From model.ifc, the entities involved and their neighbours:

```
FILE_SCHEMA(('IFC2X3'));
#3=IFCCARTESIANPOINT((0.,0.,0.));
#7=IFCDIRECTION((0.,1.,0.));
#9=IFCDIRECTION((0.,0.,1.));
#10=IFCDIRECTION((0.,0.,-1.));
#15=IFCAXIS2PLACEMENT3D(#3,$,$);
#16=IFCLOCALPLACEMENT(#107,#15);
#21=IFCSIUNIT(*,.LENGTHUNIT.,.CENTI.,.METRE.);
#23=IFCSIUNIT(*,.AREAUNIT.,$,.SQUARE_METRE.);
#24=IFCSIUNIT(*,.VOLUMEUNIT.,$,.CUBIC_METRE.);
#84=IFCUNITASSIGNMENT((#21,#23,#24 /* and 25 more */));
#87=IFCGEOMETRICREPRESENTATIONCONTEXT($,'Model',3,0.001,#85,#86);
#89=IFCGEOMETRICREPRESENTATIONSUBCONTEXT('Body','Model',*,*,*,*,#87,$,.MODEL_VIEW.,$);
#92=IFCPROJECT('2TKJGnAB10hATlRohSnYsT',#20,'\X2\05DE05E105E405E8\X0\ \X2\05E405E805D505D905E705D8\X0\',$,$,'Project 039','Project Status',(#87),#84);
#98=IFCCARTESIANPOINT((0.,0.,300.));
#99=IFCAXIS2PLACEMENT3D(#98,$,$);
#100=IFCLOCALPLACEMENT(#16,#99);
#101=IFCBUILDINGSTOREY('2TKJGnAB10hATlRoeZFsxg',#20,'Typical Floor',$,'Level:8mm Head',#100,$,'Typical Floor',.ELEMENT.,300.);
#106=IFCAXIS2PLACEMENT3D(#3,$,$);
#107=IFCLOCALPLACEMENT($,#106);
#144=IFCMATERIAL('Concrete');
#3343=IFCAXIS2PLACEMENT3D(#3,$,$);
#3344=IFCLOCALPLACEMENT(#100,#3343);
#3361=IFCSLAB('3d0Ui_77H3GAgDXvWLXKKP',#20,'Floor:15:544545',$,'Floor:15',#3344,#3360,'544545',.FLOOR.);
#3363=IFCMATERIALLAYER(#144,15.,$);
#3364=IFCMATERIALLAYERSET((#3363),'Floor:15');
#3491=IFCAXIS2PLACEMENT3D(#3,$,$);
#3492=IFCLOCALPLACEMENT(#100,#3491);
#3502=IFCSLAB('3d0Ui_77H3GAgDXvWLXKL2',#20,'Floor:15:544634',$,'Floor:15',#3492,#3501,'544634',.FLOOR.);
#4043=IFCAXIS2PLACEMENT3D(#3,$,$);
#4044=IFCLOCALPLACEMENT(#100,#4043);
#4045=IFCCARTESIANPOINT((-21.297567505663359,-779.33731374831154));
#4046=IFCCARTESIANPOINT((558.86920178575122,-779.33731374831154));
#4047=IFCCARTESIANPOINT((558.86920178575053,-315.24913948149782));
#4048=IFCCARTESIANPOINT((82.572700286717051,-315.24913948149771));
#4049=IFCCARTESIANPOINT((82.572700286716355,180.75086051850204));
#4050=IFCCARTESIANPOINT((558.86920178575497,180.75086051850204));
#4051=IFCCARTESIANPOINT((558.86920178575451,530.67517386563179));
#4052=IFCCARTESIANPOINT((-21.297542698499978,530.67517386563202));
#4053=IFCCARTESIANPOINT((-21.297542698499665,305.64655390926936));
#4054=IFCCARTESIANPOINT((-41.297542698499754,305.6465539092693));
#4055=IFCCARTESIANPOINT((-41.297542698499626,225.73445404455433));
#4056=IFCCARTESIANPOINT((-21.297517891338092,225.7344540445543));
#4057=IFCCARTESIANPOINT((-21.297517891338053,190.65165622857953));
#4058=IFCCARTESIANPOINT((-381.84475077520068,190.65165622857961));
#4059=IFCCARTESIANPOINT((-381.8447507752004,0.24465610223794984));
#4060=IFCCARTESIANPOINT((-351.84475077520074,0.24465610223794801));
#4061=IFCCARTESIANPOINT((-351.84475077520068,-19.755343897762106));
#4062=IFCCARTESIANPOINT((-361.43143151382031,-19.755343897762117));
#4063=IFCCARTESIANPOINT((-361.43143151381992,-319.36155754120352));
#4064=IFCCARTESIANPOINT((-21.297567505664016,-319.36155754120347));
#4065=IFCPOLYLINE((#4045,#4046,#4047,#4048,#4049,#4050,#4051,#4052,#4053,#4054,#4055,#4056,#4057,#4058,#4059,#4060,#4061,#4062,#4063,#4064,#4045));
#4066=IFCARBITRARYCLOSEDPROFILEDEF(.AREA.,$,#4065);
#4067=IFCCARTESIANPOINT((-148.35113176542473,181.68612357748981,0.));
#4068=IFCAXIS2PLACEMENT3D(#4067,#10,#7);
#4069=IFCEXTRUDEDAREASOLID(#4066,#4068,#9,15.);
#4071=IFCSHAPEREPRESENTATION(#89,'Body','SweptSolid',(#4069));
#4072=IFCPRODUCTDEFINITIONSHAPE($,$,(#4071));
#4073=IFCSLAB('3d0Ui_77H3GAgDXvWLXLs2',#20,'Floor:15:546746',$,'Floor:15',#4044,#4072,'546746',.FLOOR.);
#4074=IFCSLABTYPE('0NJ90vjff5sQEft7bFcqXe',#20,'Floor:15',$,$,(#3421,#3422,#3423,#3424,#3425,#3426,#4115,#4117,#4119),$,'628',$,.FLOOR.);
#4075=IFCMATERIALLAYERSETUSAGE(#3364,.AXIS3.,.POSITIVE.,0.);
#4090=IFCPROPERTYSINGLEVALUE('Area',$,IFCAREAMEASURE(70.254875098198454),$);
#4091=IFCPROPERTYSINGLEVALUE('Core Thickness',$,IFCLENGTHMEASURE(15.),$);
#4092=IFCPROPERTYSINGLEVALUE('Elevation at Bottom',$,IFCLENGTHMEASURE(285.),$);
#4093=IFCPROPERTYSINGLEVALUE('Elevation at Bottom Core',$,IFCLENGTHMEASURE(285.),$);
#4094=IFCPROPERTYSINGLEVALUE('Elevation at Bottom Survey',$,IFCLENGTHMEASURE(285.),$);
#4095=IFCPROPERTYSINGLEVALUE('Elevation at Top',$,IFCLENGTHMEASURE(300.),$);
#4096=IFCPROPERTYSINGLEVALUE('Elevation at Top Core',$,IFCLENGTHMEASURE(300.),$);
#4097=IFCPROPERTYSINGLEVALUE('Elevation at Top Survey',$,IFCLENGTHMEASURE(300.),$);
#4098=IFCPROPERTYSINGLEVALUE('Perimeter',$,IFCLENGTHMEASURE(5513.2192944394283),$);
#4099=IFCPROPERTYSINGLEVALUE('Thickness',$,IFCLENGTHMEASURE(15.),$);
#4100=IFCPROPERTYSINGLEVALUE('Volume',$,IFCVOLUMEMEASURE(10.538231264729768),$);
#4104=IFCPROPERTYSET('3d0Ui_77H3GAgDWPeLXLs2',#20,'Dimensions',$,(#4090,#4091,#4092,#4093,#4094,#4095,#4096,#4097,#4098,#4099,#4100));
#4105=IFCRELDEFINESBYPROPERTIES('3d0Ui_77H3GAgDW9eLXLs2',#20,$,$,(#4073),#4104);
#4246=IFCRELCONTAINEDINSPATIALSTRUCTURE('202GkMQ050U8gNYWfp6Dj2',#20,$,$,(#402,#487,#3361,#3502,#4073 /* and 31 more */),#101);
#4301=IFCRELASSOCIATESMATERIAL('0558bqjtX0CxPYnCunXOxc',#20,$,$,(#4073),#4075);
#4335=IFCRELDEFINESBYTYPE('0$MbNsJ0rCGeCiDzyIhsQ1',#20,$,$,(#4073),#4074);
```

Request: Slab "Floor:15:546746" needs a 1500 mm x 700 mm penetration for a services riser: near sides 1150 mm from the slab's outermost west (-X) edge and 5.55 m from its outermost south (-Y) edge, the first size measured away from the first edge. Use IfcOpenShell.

```python
import numpy as np
import ifcopenshell
import ifcopenshell.api.feature
import ifcopenshell.api.geometry
import ifcopenshell.api.pset
import ifcopenshell.api.root
import ifcopenshell.geom
import ifcopenshell.util.element
import ifcopenshell.util.placement
import ifcopenshell.util.representation
import ifcopenshell.util.shape
import ifcopenshell.util.unit

model = ifcopenshell.open("model.ifc")
unit_scale = ifcopenshell.util.unit.calculate_unit_scale(model)
area_scale = ifcopenshell.util.unit.calculate_unit_scale(model, "AREAUNIT")
volume_scale = ifcopenshell.util.unit.calculate_unit_scale(model, "VOLUMEUNIT")
settings = ifcopenshell.geom.settings()


def volume(element):
    """Net volume in cubic metres, openings subtracted."""
    shape = ifcopenshell.geom.create_shape(settings, element)
    return ifcopenshell.util.shape.get_volume(shape.geometry)


slab = model.by_guid("3d0Ui_77H3GAgDXvWLXLs2")
before = volume(slab)

# Extent in the slab's own axes, in metres. The edges named are its -X and -Y sides.
slab_shape = ifcopenshell.geom.create_shape(settings, slab)
vertices = ifcopenshell.util.shape.get_vertices(slab_shape.geometry)
x_min, y_min, bottom = vertices.min(axis=0)
top = vertices[:, 2].max()

opening = ifcopenshell.api.root.create_entity(model, ifc_class="IfcOpeningElement", name="Services riser opening")
context = ifcopenshell.util.representation.get_context(model, "Model", "Body", "MODEL_VIEW")
width, depth = 1.5, 0.7
outline = [(0.0, 0.0), (width, 0.0), (width, depth), (0.0, depth), (0.0, 0.0)]
# Overshoot both faces by 50 mm so the cut is clean.
shape = ifcopenshell.api.geometry.add_slab_representation(
    model, context=context, depth=top - bottom + 0.1, polyline=outline
)
ifcopenshell.api.geometry.assign_representation(model, product=opening, representation=shape)

matrix = ifcopenshell.util.placement.get_local_placement(slab.ObjectPlacement)
matrix[:, 3] = matrix @ np.append(np.array([x_min + 1.15, y_min + 5.55, bottom - 0.05]) / unit_scale, 1.0)
ifcopenshell.api.geometry.edit_object_placement(model, product=opening, matrix=matrix, is_si=False)
ifcopenshell.api.feature.add_feature(model, feature=opening, element=slab)

after = volume(slab)

# Update the slab's stored quantities.
pset = model.by_id(ifcopenshell.util.element.get_pset(slab, "Dimensions", should_inherit=False)["id"])
ifcopenshell.api.pset.edit_pset(model, pset=pset, properties={
    "Area": model.create_entity("IfcAreaMeasure", after / (top - bottom) / area_scale),
    "Volume": model.create_entity("IfcVolumeMeasure", after / volume_scale),
})

print(f"slab volume {before:.3f} -> {after:.3f} m3")

model.write("model_rev.ifc")
```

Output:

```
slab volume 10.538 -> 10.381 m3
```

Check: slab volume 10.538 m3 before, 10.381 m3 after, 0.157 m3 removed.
